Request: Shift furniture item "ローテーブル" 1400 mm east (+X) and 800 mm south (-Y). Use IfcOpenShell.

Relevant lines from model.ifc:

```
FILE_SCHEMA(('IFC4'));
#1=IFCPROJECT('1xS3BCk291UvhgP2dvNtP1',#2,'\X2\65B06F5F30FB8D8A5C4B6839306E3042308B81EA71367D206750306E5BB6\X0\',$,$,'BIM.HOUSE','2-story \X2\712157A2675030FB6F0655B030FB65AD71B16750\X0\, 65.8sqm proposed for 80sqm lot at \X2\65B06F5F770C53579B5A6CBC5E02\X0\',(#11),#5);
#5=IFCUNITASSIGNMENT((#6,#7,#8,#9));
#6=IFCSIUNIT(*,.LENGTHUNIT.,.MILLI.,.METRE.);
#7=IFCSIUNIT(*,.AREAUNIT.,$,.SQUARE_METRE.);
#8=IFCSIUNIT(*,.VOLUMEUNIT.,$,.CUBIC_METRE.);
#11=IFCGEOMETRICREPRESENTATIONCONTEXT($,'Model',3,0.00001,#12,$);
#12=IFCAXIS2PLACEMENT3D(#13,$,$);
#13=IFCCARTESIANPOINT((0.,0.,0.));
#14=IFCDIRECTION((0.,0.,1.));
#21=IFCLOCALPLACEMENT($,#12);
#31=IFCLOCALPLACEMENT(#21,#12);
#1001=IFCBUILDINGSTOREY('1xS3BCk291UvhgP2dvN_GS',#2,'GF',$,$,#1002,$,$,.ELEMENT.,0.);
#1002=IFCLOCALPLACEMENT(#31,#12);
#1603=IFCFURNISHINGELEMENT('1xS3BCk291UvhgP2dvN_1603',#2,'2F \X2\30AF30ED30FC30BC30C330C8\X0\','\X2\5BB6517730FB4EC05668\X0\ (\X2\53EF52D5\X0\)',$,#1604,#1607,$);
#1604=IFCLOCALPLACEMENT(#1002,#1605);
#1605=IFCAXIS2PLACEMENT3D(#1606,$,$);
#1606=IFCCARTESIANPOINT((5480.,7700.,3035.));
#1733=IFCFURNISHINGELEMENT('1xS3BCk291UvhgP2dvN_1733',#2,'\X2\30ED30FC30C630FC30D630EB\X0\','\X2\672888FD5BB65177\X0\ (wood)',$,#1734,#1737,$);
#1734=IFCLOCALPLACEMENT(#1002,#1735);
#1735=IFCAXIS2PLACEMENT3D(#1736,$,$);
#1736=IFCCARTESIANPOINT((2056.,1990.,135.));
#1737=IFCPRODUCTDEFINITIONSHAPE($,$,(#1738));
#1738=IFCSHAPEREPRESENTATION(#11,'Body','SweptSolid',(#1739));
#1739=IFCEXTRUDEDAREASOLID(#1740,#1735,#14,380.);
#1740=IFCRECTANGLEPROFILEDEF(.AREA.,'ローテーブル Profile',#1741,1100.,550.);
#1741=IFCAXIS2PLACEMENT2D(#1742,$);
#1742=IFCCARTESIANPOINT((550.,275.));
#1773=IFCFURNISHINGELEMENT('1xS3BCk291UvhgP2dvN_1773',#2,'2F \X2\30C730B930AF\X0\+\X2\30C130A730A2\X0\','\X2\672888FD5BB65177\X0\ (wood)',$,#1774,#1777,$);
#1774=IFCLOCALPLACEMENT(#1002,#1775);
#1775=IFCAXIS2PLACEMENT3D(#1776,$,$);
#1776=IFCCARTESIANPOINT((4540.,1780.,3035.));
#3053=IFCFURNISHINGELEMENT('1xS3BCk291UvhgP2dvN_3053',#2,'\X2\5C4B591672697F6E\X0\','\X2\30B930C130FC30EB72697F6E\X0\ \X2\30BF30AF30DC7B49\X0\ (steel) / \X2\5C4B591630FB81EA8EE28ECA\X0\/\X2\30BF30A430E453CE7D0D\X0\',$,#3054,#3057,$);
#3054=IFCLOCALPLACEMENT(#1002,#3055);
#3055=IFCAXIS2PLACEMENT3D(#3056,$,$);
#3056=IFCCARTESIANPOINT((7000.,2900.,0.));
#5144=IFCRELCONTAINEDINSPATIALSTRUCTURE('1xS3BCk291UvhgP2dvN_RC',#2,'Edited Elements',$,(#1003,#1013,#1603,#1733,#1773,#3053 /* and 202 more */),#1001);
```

```python
import ifcopenshell
import ifcopenshell.api.geometry
import ifcopenshell.util.placement
import ifcopenshell.util.unit

model = ifcopenshell.open("model.ifc")
unit_scale = ifcopenshell.util.unit.calculate_unit_scale(model)

item = model.by_guid("1xS3BCk291UvhgP2dvN_1733")
matrix = ifcopenshell.util.placement.get_local_placement(item.ObjectPlacement)
matrix[0, 3] += 1.4 / unit_scale
matrix[1, 3] -= 0.8 / unit_scale
ifcopenshell.api.geometry.edit_object_placement(model, product=item, matrix=matrix, is_si=False)

print(ifcopenshell.util.placement.get_local_placement(item.ObjectPlacement).round(3) + 0.0)

model.write("model_updated.ifc")
```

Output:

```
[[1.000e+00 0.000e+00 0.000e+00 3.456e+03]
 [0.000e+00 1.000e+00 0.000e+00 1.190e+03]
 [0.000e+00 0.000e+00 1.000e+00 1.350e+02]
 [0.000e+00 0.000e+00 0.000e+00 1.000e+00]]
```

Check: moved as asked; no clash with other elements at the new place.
